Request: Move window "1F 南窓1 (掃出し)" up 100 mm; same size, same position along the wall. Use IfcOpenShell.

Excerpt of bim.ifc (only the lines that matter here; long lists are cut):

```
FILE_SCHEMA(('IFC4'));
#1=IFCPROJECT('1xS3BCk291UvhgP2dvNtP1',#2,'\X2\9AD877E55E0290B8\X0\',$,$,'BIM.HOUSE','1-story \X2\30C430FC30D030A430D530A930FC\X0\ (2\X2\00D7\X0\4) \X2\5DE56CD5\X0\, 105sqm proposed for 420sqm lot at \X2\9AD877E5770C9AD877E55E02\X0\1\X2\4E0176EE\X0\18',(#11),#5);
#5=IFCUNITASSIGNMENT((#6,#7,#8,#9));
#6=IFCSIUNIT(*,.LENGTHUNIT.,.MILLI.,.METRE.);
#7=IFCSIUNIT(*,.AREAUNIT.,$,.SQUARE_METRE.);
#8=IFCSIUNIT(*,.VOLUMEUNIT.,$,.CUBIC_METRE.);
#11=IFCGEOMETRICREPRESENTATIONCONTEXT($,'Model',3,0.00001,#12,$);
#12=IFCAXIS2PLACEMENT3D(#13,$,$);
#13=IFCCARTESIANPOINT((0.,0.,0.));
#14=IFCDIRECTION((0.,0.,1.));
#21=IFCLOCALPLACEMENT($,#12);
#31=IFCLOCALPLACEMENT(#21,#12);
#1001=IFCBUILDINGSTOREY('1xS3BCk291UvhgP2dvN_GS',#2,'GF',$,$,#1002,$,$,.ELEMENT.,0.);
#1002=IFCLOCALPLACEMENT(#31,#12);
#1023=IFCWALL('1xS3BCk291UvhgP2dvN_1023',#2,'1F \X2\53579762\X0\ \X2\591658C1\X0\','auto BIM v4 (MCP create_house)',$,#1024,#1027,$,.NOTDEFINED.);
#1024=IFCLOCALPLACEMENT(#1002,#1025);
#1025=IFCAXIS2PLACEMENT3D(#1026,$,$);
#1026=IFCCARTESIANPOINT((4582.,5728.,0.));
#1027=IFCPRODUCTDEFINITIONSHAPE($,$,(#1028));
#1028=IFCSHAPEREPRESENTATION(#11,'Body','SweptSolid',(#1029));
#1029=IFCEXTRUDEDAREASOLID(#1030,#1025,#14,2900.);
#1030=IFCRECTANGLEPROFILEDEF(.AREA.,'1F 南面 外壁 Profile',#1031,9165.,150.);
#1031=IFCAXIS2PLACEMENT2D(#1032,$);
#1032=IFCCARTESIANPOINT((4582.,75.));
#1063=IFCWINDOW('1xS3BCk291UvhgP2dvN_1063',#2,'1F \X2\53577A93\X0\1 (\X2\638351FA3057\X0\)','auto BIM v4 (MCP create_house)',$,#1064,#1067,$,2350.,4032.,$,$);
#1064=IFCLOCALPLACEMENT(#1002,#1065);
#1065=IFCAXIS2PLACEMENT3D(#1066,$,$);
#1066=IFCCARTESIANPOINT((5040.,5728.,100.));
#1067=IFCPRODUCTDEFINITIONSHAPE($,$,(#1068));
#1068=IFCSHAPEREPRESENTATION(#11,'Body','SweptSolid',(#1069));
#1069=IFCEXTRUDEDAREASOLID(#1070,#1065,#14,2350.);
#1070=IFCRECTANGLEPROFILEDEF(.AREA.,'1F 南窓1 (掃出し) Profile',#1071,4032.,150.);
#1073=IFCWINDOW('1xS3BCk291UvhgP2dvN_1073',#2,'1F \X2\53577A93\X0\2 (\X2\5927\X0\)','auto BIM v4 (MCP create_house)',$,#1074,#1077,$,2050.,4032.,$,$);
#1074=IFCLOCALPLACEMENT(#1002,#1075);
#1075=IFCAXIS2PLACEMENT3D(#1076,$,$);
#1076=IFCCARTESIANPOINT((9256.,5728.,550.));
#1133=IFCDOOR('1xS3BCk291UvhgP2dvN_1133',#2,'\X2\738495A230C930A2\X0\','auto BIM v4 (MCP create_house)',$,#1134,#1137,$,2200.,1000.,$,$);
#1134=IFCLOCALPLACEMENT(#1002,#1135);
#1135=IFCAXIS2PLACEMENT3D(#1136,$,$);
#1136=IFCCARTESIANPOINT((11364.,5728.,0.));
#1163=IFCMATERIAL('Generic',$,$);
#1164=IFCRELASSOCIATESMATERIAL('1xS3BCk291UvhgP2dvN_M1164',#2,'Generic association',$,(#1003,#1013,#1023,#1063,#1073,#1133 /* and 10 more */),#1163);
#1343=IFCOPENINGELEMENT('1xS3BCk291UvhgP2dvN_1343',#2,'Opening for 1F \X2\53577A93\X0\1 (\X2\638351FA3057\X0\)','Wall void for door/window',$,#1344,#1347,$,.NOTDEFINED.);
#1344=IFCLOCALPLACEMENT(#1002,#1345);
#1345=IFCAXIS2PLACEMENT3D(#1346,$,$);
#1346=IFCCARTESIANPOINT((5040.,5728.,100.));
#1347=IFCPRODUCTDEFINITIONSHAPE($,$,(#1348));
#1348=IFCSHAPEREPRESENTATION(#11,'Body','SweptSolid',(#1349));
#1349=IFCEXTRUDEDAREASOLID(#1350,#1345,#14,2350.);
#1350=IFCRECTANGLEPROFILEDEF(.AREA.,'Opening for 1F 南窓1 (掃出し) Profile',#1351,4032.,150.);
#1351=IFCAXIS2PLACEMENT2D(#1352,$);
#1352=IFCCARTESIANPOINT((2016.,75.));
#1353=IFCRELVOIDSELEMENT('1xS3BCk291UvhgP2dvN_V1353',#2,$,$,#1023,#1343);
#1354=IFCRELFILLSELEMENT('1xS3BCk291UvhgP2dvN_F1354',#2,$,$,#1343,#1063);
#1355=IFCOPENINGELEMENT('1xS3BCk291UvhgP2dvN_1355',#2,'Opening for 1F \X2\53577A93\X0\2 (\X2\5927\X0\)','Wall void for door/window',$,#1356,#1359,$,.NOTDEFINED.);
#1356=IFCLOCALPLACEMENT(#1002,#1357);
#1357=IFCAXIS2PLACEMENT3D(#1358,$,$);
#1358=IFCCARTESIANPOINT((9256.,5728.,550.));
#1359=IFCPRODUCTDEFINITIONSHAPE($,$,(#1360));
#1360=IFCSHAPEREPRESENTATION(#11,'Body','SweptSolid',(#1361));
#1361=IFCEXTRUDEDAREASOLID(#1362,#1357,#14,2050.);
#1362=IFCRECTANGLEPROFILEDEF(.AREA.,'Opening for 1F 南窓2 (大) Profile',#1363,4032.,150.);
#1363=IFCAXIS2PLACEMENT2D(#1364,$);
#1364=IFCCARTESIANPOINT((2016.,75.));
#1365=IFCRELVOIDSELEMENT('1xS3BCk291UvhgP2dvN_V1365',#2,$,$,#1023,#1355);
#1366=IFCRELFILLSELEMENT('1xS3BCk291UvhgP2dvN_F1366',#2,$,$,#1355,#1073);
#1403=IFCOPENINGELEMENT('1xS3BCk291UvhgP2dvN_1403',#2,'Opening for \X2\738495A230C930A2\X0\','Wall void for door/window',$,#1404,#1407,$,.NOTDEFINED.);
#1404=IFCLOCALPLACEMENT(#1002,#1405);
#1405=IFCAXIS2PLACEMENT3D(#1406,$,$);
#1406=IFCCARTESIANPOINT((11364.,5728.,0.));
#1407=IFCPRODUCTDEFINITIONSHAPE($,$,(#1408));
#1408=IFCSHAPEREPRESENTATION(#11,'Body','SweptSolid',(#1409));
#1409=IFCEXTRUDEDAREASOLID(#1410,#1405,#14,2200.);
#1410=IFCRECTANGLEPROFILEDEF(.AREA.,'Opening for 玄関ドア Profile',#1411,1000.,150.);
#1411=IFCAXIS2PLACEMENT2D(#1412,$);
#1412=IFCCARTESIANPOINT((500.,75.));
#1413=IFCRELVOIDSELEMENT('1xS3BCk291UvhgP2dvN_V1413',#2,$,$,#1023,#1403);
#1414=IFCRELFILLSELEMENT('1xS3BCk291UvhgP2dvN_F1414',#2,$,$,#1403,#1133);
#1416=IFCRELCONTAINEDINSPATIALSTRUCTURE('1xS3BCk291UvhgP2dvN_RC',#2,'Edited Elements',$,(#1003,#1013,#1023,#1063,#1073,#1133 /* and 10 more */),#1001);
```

```python
import numpy as np
import ifcopenshell
import ifcopenshell.api.geometry
import ifcopenshell.util.placement
import ifcopenshell.util.unit

model = ifcopenshell.open("bim.ifc")
unit_scale = ifcopenshell.util.unit.calculate_unit_scale(model)

window = model.by_guid("1xS3BCk291UvhgP2dvN_1063")
opening = window.FillsVoids[0].RelatingOpeningElement
dz = 0.1 / unit_scale

shift = np.array([0.0, 0.0, dz])
# The window is not placed relative to its opening, so move both.
for product in (opening, window):
    matrix = ifcopenshell.util.placement.get_local_placement(product.ObjectPlacement)
    matrix[:3, 3] += shift
    ifcopenshell.api.geometry.edit_object_placement(model, product=product, matrix=matrix, is_si=False)

print(f"moved by {dz * unit_scale:+.3f} m")

model.write("bim_updated.ifc")
```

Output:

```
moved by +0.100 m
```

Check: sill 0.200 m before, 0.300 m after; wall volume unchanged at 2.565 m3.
